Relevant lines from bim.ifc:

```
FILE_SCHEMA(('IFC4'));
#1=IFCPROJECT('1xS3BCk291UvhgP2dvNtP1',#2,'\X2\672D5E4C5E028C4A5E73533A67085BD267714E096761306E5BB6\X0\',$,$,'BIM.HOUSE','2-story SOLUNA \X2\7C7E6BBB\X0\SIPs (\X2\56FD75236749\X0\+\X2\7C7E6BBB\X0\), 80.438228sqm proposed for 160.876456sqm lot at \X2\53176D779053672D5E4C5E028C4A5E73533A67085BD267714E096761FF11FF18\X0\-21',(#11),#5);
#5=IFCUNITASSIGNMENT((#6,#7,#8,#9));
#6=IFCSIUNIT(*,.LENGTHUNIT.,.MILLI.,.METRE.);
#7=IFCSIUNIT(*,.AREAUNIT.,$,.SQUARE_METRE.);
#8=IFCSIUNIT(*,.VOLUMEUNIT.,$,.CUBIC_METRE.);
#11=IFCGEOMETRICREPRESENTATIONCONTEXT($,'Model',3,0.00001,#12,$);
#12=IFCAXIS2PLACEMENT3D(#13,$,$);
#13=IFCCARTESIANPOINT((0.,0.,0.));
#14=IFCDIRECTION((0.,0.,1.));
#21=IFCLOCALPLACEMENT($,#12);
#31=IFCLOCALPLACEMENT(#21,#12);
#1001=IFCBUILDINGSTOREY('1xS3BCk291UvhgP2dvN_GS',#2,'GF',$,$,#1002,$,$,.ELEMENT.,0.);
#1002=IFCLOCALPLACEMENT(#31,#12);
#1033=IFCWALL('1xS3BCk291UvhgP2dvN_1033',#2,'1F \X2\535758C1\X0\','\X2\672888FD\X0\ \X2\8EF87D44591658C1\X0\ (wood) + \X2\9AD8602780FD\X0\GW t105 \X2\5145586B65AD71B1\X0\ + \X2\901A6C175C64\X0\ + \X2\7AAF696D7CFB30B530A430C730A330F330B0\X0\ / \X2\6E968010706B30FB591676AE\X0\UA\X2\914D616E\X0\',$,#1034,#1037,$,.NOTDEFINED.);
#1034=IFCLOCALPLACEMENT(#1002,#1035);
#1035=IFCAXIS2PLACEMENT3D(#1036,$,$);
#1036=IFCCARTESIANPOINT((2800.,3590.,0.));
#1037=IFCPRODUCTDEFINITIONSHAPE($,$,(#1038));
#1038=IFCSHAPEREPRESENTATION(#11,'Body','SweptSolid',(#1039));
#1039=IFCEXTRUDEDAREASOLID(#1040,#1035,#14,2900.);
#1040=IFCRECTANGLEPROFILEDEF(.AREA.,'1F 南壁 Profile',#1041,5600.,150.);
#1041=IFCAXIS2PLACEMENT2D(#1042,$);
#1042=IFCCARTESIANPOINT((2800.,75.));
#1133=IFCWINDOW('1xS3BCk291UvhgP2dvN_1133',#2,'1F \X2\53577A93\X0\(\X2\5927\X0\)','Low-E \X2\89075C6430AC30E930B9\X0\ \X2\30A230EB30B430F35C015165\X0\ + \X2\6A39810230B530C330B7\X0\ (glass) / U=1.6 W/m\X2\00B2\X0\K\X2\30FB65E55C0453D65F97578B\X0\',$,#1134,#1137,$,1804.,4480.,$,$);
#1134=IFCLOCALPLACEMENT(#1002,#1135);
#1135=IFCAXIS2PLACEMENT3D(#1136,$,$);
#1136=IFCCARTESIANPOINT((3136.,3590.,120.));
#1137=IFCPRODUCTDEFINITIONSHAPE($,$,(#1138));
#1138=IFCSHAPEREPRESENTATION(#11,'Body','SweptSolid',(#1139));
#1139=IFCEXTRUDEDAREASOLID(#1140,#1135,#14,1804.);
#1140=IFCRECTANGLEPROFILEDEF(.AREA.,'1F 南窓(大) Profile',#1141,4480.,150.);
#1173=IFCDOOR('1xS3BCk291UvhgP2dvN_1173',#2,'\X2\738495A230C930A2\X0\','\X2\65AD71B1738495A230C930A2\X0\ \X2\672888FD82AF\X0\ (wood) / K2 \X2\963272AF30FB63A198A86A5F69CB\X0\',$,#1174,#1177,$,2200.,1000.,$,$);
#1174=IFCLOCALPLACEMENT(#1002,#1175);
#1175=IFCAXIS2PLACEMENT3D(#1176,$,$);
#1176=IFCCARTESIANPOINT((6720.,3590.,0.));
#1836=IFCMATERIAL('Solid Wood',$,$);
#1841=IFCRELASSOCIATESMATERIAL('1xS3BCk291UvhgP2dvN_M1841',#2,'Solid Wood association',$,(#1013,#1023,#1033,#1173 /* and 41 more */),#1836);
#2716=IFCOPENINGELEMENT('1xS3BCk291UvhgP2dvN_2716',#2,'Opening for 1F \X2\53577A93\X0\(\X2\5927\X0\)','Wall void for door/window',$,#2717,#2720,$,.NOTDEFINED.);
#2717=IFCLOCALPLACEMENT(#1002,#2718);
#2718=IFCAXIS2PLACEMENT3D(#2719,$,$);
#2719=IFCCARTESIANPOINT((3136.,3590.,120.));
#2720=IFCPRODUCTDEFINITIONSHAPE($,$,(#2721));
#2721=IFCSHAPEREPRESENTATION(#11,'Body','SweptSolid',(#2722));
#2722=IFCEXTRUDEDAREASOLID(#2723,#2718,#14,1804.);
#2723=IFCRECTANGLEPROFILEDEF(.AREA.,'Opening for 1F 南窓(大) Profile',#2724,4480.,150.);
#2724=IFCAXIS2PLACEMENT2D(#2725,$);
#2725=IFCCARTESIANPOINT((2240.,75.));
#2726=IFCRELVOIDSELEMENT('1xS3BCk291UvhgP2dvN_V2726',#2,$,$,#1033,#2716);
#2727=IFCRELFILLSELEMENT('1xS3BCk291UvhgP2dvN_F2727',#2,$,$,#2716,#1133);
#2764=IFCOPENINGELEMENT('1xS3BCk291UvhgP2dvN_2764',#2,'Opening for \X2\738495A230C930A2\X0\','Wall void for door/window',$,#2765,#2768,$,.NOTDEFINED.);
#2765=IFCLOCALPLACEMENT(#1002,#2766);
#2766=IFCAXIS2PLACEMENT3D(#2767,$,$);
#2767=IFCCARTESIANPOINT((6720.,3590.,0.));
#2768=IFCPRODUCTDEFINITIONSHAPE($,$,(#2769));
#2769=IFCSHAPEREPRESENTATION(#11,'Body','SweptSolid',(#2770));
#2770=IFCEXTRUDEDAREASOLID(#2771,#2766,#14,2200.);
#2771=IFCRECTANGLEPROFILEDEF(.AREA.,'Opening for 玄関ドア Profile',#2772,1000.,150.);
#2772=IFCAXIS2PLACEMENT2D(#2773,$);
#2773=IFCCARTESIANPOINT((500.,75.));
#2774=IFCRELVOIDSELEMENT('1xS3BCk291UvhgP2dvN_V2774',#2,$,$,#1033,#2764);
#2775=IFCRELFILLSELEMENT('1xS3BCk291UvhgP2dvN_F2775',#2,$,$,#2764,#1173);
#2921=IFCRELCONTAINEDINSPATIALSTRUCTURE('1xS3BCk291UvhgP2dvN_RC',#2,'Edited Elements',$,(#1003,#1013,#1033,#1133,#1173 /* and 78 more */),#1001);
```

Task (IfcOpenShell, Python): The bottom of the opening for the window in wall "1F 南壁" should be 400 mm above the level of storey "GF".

```python
import numpy as np
import ifcopenshell
import ifcopenshell.api.geometry
import ifcopenshell.geom
import ifcopenshell.util.element
import ifcopenshell.util.placement
import ifcopenshell.util.shape
import ifcopenshell.util.unit

model = ifcopenshell.open("bim.ifc")
unit_scale = ifcopenshell.util.unit.calculate_unit_scale(model)

window = model.by_guid("1xS3BCk291UvhgP2dvN_1133")
opening = window.FillsVoids[0].RelatingOpeningElement
storey = ifcopenshell.util.element.get_container(window, ifc_class="IfcBuildingStorey")
level = ifcopenshell.util.placement.get_local_placement(storey.ObjectPlacement)[2, 3]

# The opening's origin need not be at the sill, so measure its lowest point.
shape = ifcopenshell.geom.create_shape(ifcopenshell.geom.settings(), opening)
bottom = ifcopenshell.util.shape.get_shape_bottom_elevation(shape, shape.geometry) / unit_scale
dz = level + 0.4 / unit_scale - bottom

shift = np.array([0.0, 0.0, dz])
# The window is not placed relative to its opening, so move both.
for product in (opening, window):
    matrix = ifcopenshell.util.placement.get_local_placement(product.ObjectPlacement)
    matrix[:3, 3] += shift
    ifcopenshell.api.geometry.edit_object_placement(model, product=product, matrix=matrix, is_si=False)

print(f"moved by {dz * unit_scale:+.3f} m")

model.write("bim_v2.ifc")
```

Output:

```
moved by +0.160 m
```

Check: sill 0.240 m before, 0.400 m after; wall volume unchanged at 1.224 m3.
